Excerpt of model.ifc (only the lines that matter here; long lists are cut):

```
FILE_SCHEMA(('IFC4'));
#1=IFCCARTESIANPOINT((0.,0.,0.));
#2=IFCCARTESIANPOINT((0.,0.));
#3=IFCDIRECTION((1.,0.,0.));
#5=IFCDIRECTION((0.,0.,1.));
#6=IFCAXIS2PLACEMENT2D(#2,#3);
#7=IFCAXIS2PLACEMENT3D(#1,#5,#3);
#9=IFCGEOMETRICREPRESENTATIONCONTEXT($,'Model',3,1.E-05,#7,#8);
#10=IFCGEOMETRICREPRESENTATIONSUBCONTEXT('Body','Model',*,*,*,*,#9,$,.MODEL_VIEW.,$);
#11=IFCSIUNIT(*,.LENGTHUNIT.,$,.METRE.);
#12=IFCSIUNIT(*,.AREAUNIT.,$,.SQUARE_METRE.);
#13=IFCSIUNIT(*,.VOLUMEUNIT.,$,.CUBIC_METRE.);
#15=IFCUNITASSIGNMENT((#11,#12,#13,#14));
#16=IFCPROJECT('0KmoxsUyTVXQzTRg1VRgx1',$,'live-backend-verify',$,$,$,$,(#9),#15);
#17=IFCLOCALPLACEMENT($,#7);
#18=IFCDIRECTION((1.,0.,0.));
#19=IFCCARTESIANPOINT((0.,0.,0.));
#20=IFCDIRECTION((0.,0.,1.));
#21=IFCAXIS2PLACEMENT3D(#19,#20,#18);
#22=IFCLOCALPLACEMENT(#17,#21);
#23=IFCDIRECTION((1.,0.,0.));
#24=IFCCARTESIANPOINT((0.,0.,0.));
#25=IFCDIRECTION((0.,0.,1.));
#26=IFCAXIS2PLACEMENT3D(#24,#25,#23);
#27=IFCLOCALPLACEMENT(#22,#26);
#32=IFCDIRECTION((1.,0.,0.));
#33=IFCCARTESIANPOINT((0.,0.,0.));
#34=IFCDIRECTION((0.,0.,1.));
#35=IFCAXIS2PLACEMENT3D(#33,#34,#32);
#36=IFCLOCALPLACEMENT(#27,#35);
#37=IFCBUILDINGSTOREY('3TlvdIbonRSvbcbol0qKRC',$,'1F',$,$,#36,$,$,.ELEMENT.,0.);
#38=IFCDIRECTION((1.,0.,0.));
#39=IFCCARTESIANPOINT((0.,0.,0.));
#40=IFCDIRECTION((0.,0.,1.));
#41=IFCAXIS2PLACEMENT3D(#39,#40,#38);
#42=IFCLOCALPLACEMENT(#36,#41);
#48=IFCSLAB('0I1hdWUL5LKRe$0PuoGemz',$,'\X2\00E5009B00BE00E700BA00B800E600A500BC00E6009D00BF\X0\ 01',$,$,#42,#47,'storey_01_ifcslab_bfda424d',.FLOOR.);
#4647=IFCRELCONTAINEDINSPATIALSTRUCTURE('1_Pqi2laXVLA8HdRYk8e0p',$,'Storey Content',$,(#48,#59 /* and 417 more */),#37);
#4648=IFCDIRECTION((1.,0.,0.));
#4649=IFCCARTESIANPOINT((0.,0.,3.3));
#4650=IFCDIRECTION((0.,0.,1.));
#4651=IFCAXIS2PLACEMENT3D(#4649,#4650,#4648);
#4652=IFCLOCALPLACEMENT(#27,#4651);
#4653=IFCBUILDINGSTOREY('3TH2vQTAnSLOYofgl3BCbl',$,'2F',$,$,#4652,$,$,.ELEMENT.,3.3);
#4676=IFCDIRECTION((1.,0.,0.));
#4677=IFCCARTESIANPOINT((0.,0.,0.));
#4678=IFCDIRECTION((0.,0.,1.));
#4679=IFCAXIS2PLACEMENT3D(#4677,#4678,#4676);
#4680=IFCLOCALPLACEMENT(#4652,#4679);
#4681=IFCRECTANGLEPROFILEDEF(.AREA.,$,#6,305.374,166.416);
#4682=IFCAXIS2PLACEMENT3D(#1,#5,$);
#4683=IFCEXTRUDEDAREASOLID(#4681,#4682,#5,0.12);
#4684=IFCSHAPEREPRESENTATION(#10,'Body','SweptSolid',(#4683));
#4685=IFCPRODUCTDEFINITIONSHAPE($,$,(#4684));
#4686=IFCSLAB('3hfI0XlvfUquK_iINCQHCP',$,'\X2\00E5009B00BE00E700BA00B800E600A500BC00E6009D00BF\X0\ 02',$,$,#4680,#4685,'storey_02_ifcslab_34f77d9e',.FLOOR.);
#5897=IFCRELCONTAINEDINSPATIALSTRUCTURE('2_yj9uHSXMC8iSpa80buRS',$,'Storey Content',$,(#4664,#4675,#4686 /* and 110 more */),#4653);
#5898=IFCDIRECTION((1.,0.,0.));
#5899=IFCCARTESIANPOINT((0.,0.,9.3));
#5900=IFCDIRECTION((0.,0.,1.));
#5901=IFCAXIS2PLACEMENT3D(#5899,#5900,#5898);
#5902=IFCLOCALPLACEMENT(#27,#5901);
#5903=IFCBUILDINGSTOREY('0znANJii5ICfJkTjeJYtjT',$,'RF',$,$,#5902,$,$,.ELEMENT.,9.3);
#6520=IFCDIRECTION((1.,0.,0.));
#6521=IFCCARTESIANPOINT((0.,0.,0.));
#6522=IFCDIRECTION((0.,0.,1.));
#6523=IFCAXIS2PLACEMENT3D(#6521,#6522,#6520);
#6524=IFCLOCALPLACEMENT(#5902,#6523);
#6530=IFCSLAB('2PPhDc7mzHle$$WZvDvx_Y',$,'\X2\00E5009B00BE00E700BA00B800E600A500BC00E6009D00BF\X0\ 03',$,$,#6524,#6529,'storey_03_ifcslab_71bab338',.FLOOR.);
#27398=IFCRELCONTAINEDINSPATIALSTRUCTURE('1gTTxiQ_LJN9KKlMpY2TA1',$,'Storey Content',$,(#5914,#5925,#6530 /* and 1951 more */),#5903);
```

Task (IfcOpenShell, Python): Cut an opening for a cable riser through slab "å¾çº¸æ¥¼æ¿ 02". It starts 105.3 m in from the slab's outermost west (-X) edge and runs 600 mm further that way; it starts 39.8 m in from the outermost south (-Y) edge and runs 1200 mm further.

```python
import numpy as np
import ifcopenshell
import ifcopenshell.api.feature
import ifcopenshell.api.geometry
import ifcopenshell.api.root
import ifcopenshell.geom
import ifcopenshell.util.placement
import ifcopenshell.util.representation
import ifcopenshell.util.shape
import ifcopenshell.util.unit

model = ifcopenshell.open("model.ifc")
unit_scale = ifcopenshell.util.unit.calculate_unit_scale(model)
settings = ifcopenshell.geom.settings()


def volume(element):
    """Net volume in cubic metres, openings subtracted."""
    shape = ifcopenshell.geom.create_shape(settings, element)
    return ifcopenshell.util.shape.get_volume(shape.geometry)


slab = model.by_guid("3hfI0XlvfUquK_iINCQHCP")
before = volume(slab)

# Extent in the slab's own axes, in metres. The edges named are its -X and -Y sides.
slab_shape = ifcopenshell.geom.create_shape(settings, slab)
vertices = ifcopenshell.util.shape.get_vertices(slab_shape.geometry)
x_min, y_min, bottom = vertices.min(axis=0)
top = vertices[:, 2].max()

opening = ifcopenshell.api.root.create_entity(model, ifc_class="IfcOpeningElement", name="Cable riser opening", predefined_type="OPENING")
context = ifcopenshell.util.representation.get_context(model, "Model", "Body", "MODEL_VIEW")
width, depth = 0.6, 1.2
outline = [(0.0, 0.0), (width, 0.0), (width, depth), (0.0, depth), (0.0, 0.0)]
# Overshoot both faces by 50 mm so the cut is clean.
shape = ifcopenshell.api.geometry.add_slab_representation(
    model, context=context, depth=top - bottom + 0.1, polyline=outline
)
ifcopenshell.api.geometry.assign_representation(model, product=opening, representation=shape)

matrix = ifcopenshell.util.placement.get_local_placement(slab.ObjectPlacement)
matrix[:, 3] = matrix @ np.append(np.array([x_min + 105.3, y_min + 39.8, bottom - 0.05]) / unit_scale, 1.0)
ifcopenshell.api.geometry.edit_object_placement(model, product=opening, matrix=matrix, is_si=False)
ifcopenshell.api.feature.add_feature(model, feature=opening, element=slab)

after = volume(slab)

print(f"slab volume {before:.3f} -> {after:.3f} m3")

model.write("model_rev.ifc")
```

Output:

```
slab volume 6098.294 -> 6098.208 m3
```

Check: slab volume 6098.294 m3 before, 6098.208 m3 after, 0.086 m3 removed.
